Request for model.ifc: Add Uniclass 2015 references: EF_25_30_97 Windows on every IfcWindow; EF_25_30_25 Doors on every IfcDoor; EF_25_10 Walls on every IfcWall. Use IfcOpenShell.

First a look at what the model holds.

```python
import ifcopenshell

model = ifcopenshell.open("model.ifc")
print(model.schema)
print("classifications:", [c.Name for c in model.by_type("IfcClassification")])
for ifc_class in ("IfcDoor", "IfcRoof", "IfcStair", "IfcWall", "IfcWindow"):
    print(ifc_class, len(model.by_type(ifc_class)))
```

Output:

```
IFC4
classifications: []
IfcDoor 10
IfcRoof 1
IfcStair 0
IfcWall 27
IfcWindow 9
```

```python
import ifcopenshell
import ifcopenshell.api.classification

model = ifcopenshell.open("model.ifc")

system = ifcopenshell.api.classification.add_classification(model, classification="Uniclass 2015")

codes = {
    "IfcWindow": ("EF_25_30_97", "Windows"),
    "IfcDoor": ("EF_25_30_25", "Doors"),
    "IfcWall": ("EF_25_10", "Walls"),
}
for ifc_class, (code, name) in codes.items():
    products = model.by_type(ifc_class)
    ifcopenshell.api.classification.add_reference(
        model, products=products, classification=system, identification=code, name=name
    )
    print(code, len(products))

model.write("model_edited.ifc")
```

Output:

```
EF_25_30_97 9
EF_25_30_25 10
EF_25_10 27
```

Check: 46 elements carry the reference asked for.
